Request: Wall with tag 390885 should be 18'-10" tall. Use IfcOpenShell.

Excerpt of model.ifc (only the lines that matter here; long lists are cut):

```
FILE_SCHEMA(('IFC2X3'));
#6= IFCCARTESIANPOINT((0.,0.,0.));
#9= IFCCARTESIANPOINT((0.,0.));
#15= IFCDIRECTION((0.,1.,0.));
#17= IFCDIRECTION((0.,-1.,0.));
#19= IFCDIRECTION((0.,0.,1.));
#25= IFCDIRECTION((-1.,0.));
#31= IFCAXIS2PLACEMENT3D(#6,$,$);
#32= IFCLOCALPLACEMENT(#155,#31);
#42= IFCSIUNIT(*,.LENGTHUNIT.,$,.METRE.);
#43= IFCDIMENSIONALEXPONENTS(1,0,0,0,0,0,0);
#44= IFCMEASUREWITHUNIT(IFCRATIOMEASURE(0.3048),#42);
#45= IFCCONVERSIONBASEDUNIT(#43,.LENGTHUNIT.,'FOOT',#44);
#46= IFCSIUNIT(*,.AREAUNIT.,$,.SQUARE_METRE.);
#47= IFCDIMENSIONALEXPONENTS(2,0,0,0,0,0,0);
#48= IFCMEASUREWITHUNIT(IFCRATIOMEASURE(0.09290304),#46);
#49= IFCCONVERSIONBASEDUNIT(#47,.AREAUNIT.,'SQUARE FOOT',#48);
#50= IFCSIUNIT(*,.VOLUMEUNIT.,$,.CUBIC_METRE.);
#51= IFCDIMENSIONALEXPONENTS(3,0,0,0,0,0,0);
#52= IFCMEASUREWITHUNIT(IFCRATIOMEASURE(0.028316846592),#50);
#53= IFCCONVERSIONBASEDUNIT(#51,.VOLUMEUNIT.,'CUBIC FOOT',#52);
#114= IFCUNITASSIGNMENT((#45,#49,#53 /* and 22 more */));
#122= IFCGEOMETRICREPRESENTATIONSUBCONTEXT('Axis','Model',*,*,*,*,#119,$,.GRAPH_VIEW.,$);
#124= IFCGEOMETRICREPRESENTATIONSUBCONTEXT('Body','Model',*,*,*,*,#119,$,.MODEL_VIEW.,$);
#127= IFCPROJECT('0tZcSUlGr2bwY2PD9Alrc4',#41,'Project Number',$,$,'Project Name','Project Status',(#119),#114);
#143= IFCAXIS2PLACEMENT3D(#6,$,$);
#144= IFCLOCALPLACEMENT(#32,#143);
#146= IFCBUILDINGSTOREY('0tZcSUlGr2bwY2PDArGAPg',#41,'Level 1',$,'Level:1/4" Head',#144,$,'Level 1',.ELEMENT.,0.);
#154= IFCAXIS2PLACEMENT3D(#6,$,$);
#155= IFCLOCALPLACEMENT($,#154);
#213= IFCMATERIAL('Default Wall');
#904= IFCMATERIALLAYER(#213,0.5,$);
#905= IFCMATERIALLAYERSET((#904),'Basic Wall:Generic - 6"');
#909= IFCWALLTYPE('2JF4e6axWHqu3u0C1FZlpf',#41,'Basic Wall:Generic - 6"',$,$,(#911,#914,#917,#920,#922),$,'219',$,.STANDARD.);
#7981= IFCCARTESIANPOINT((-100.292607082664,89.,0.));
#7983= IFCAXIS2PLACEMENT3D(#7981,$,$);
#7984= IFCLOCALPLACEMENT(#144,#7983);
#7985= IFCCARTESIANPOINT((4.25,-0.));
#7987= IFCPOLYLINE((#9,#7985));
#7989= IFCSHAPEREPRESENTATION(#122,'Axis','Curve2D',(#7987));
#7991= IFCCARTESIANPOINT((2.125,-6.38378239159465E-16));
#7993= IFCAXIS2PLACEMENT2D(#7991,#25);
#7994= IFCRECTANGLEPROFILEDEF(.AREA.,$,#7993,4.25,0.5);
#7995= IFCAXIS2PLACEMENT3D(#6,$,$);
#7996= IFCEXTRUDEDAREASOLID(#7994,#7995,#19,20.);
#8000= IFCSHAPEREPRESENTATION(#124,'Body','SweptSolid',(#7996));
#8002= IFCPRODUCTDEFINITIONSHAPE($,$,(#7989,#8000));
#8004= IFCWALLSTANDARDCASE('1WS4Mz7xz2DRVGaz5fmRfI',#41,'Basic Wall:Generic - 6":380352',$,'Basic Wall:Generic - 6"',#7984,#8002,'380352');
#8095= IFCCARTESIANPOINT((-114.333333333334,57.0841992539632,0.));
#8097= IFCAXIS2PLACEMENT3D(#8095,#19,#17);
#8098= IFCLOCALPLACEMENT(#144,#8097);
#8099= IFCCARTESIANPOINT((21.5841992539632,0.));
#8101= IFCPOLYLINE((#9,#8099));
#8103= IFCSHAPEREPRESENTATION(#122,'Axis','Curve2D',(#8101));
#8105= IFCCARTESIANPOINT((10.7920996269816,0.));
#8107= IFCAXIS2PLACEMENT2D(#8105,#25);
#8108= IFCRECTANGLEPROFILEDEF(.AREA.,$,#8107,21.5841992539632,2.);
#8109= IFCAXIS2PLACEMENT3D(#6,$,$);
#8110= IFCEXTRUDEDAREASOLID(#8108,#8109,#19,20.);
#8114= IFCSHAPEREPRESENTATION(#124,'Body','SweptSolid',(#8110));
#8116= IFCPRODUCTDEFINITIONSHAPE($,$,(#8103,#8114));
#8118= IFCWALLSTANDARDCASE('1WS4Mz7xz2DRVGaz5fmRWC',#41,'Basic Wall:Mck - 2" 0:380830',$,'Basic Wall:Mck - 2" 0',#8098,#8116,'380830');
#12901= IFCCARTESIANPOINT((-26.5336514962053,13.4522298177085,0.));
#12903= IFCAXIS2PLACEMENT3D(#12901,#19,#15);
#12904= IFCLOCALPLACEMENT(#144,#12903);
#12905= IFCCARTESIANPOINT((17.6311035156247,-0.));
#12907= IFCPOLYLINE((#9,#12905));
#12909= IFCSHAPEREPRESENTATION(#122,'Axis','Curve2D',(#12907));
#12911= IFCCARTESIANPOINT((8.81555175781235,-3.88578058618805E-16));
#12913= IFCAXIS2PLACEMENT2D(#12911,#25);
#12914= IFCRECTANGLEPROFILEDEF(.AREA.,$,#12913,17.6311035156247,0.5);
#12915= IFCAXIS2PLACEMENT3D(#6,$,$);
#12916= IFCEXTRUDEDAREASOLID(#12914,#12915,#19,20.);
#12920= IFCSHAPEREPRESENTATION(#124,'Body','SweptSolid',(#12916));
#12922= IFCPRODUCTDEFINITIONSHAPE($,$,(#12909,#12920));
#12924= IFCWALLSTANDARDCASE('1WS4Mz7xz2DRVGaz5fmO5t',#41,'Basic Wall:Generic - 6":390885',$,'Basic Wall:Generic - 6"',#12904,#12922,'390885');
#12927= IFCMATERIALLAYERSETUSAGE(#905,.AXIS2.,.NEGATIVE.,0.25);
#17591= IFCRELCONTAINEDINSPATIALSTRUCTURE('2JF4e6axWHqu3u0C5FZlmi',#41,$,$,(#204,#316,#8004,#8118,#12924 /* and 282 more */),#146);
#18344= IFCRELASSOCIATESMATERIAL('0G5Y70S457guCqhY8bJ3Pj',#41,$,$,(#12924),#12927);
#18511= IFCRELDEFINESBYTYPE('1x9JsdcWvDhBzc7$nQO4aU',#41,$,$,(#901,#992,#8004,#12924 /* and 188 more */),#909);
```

```python
import ifcopenshell
import ifcopenshell.geom
import ifcopenshell.util.representation
import ifcopenshell.util.shape
import ifcopenshell.util.unit

model = ifcopenshell.open("model.ifc")
unit_scale = ifcopenshell.util.unit.calculate_unit_scale(model)
settings = ifcopenshell.geom.settings()


def volume(element):
    """Net volume in cubic metres, openings subtracted."""
    shape = ifcopenshell.geom.create_shape(settings, element)
    return ifcopenshell.util.shape.get_volume(shape.geometry)


wall = model.by_guid("1WS4Mz7xz2DRVGaz5fmO5t")
before = volume(wall)

body = ifcopenshell.util.representation.get_representation(wall, "Model", "Body")
solid = body.Items[0]
old_height = solid.Depth
solid.Depth = 226 * 0.0254 / unit_scale
after = volume(wall)

print(f"height {old_height:g} -> {solid.Depth:g}, volume {before:.3f} -> {after:.3f} m3")

model.write("model_rev.ifc")
```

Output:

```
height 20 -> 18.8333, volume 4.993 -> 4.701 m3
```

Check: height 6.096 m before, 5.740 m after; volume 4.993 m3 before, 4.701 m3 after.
